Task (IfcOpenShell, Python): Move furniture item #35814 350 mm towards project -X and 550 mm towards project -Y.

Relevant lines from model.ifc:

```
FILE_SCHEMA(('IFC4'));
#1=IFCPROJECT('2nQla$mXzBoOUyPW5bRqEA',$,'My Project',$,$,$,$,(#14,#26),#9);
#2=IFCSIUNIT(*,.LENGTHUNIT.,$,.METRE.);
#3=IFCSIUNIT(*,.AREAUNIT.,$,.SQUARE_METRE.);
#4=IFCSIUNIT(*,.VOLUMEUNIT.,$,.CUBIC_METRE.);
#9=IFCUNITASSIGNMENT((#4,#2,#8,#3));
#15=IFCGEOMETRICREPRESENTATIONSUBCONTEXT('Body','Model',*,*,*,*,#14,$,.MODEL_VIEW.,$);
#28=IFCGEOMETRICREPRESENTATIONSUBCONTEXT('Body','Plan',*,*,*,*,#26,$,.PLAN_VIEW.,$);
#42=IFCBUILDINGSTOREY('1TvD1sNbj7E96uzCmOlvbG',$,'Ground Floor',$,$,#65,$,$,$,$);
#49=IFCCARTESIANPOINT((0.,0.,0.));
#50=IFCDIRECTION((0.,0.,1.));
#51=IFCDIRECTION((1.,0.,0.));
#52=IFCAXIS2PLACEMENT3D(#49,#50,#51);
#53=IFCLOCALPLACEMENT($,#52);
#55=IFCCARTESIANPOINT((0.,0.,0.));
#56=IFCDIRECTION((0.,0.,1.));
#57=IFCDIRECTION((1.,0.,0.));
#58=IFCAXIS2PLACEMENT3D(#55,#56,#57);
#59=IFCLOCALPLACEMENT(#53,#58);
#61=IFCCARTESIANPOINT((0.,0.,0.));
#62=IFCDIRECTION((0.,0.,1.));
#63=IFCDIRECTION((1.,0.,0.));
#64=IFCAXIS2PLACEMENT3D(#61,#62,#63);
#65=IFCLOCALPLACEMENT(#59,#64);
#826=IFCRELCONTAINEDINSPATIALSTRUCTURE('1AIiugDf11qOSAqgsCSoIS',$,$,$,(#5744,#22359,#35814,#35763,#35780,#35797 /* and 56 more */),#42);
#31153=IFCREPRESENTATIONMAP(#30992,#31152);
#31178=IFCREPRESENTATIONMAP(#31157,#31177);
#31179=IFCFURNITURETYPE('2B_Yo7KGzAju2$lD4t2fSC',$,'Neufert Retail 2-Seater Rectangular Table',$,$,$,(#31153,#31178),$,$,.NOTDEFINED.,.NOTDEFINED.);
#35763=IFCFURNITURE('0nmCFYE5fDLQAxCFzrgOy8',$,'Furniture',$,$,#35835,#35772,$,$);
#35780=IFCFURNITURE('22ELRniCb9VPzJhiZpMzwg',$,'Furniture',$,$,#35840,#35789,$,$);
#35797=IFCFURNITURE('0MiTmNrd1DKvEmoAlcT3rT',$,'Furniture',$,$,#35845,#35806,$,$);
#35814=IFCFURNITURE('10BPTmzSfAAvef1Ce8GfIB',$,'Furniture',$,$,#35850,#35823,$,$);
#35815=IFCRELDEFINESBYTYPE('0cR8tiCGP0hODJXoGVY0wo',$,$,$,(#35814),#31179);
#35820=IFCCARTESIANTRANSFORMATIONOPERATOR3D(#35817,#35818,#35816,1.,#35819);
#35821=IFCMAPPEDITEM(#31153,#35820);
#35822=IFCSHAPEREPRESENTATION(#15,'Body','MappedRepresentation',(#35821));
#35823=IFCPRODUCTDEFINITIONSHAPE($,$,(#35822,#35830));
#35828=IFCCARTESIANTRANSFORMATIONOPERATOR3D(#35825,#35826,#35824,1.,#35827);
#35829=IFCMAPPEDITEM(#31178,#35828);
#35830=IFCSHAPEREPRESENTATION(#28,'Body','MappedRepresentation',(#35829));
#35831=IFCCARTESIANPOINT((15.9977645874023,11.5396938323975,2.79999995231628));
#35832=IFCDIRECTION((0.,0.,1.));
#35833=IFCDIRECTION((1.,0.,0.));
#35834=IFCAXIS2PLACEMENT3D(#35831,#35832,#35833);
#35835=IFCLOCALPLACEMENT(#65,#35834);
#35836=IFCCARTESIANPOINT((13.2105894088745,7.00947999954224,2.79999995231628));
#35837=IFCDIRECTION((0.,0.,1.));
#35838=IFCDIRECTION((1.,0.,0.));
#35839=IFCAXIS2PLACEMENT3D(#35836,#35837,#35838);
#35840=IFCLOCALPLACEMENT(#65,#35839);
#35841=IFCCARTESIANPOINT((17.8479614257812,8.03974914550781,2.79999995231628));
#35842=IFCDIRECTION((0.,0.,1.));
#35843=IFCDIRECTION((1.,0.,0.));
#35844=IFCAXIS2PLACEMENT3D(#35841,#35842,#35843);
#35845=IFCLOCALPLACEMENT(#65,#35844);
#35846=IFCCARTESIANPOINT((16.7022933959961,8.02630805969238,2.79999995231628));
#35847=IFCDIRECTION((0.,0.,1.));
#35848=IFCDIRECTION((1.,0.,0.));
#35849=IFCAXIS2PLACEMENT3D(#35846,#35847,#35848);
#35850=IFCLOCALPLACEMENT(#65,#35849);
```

```python
import ifcopenshell
import ifcopenshell.api.geometry
import ifcopenshell.util.placement
import ifcopenshell.util.unit

model = ifcopenshell.open("model.ifc")
unit_scale = ifcopenshell.util.unit.calculate_unit_scale(model)

item = model.by_id(35814)
matrix = ifcopenshell.util.placement.get_local_placement(item.ObjectPlacement)
matrix[0, 3] -= 0.35 / unit_scale
matrix[1, 3] -= 0.55 / unit_scale
ifcopenshell.api.geometry.edit_object_placement(model, product=item, matrix=matrix, is_si=False)

print(ifcopenshell.util.placement.get_local_placement(item.ObjectPlacement).round(3) + 0.0)

model.write("model_updated.ifc")
```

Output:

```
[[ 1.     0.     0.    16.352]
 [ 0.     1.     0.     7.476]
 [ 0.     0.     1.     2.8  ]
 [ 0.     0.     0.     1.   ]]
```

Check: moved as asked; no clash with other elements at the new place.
